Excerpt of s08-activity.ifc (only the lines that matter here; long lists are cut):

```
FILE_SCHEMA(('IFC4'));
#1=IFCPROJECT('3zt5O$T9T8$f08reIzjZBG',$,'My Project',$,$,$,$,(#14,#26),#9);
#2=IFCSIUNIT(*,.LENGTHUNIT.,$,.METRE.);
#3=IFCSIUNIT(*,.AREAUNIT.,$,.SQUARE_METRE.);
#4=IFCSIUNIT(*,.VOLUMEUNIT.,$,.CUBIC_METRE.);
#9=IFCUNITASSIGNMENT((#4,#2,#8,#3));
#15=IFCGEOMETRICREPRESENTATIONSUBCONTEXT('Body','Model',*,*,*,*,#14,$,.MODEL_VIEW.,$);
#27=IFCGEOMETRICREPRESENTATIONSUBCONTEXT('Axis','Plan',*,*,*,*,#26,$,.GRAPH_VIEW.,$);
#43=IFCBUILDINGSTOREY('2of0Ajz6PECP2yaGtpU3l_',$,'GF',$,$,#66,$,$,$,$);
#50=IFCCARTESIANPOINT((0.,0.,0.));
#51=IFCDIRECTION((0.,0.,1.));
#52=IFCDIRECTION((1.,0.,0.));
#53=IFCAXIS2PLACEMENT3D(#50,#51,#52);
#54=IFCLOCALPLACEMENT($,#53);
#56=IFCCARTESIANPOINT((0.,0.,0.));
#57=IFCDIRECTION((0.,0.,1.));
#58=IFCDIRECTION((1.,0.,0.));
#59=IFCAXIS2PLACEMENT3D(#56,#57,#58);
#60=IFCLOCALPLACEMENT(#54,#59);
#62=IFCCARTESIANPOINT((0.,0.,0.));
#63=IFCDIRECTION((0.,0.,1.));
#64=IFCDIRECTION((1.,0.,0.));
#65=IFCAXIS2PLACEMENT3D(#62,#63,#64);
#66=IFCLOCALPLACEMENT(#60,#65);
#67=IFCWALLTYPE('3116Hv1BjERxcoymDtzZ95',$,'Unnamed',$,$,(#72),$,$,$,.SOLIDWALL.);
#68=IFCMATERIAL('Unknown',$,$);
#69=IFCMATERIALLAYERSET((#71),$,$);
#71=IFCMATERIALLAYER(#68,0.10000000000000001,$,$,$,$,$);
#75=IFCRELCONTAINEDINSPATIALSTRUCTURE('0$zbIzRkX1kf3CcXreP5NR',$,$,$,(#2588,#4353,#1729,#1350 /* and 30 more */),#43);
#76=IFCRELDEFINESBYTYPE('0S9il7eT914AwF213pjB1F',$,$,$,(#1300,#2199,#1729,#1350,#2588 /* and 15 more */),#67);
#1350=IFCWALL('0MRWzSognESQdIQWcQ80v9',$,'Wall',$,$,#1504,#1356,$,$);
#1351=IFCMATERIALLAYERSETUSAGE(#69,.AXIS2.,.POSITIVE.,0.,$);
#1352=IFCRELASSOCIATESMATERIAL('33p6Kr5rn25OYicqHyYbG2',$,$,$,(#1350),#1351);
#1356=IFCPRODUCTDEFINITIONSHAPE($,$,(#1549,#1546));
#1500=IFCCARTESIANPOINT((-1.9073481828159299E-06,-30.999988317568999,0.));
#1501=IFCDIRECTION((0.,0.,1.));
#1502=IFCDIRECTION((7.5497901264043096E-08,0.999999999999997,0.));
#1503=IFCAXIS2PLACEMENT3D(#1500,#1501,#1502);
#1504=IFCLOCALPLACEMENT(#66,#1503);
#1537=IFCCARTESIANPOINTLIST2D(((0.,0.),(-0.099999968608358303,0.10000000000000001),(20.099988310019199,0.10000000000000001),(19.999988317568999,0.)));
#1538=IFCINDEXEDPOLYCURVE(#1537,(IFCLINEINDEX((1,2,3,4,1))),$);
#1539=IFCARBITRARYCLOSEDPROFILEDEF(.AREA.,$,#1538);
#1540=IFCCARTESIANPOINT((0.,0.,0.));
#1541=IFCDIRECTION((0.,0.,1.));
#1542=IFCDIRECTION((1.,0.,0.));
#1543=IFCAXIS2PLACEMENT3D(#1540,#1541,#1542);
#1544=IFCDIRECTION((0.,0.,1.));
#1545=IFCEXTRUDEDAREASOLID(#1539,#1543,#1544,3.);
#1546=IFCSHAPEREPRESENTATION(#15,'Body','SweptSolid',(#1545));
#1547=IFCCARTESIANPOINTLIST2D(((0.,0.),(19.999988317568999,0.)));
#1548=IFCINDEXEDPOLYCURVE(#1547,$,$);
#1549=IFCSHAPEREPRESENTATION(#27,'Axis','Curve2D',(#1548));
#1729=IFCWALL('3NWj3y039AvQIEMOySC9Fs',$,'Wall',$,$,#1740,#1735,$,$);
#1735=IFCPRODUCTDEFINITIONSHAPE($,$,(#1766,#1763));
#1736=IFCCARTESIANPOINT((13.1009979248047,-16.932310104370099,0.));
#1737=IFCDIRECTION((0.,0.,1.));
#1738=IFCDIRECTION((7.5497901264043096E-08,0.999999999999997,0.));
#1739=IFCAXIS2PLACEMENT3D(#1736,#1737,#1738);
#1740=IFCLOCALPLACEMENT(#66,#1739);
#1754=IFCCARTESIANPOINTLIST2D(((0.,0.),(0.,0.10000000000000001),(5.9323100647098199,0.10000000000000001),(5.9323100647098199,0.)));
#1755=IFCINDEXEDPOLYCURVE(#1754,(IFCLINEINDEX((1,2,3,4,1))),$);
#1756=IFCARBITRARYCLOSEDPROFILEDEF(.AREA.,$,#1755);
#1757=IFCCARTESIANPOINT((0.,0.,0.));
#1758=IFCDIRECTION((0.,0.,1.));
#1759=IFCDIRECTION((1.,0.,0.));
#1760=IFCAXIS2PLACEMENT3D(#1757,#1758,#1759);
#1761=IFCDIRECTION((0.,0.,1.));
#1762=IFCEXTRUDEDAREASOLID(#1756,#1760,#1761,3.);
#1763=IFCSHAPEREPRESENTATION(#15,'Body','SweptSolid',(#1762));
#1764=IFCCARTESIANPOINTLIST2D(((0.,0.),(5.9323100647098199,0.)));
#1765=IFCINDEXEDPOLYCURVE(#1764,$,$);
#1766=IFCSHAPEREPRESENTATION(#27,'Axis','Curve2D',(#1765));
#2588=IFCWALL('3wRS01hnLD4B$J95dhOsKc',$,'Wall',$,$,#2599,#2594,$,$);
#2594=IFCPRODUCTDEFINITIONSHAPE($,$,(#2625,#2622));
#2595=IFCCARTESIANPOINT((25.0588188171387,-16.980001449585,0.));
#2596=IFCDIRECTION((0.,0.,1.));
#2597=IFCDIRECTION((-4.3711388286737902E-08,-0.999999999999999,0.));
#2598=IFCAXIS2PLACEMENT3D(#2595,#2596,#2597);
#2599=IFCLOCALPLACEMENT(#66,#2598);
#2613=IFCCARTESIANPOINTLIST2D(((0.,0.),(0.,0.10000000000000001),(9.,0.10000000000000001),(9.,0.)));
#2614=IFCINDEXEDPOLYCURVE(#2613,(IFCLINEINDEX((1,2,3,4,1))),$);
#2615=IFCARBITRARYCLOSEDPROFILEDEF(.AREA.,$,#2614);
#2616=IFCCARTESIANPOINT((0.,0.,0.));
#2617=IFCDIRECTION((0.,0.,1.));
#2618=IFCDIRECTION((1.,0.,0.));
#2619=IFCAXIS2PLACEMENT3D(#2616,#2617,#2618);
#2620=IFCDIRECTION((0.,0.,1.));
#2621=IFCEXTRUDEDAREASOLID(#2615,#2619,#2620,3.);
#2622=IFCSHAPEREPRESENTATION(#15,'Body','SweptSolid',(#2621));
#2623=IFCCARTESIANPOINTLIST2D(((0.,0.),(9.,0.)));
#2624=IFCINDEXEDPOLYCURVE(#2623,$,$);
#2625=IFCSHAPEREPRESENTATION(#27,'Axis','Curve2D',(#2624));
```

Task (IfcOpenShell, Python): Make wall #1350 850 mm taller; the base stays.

```python
import ifcopenshell
import ifcopenshell.geom
import ifcopenshell.util.representation
import ifcopenshell.util.shape

model = ifcopenshell.open("s08-activity.ifc")
settings = ifcopenshell.geom.settings()


def volume(element):
    """Net volume in cubic metres, openings subtracted."""
    shape = ifcopenshell.geom.create_shape(settings, element)
    return ifcopenshell.util.shape.get_volume(shape.geometry)


wall = model.by_guid("0MRWzSognESQdIQWcQ80v9")
before = volume(wall)

body = ifcopenshell.util.representation.get_representation(wall, "Model", "Body")
solid = body.Items[0]
old_height = solid.Depth
solid.Depth += 0.85
after = volume(wall)

print(f"height {old_height:g} -> {solid.Depth:g}, volume {before:.3f} -> {after:.3f} m3")

model.write("s08-activity_rev.ifc")
```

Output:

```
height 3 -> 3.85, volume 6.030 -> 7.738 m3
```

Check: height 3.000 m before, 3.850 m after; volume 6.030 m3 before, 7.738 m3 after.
